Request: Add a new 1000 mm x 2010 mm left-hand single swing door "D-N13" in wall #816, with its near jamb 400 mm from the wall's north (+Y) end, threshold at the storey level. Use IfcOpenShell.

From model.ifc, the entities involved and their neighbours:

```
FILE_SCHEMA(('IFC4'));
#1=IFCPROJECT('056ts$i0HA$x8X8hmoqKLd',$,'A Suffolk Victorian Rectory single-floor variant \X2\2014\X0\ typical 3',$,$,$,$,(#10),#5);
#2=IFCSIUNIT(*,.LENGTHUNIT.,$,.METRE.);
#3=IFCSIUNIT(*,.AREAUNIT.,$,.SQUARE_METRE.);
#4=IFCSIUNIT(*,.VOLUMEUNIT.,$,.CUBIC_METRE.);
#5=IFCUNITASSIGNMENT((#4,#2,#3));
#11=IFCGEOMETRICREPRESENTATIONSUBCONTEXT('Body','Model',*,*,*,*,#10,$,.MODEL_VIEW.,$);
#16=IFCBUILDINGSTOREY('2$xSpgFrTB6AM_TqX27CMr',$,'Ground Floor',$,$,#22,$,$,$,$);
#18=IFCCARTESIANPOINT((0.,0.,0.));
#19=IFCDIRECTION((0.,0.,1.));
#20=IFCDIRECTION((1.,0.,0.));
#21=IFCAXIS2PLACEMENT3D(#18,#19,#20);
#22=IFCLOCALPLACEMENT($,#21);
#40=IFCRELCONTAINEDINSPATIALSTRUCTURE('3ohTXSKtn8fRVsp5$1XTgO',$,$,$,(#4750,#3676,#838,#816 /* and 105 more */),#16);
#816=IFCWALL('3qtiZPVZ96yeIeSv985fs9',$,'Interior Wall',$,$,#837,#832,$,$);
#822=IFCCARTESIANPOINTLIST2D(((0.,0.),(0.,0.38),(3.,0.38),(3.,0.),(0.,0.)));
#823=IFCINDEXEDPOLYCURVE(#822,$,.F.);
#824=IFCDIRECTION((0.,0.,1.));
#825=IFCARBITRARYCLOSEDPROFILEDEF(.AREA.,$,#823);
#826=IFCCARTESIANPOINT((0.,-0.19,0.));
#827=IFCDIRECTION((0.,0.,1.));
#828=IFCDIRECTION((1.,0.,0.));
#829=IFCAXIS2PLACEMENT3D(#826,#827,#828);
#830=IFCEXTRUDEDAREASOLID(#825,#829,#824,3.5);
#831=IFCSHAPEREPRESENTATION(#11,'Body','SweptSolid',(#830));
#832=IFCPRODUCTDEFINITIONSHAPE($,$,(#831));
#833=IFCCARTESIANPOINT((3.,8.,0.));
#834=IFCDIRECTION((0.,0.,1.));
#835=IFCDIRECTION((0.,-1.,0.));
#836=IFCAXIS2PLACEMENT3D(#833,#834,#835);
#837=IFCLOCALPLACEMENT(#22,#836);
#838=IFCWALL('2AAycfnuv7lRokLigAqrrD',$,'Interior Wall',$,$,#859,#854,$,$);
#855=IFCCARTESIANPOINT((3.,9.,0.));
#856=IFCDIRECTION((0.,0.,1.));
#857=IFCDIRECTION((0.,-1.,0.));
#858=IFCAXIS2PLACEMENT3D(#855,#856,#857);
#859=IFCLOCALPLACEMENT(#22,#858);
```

```python
import numpy as np
import ifcopenshell
import ifcopenshell.api.feature
import ifcopenshell.api.geometry
import ifcopenshell.api.root
import ifcopenshell.api.spatial
import ifcopenshell.geom
import ifcopenshell.util.element
import ifcopenshell.util.placement
import ifcopenshell.util.representation
import ifcopenshell.util.shape
import ifcopenshell.util.unit

model = ifcopenshell.open("model.ifc")
unit_scale = ifcopenshell.util.unit.calculate_unit_scale(model)
settings = ifcopenshell.geom.settings()


def volume(element):
    """Net volume in cubic metres, openings subtracted."""
    shape = ifcopenshell.geom.create_shape(settings, element)
    return ifcopenshell.util.shape.get_volume(shape.geometry)


wall = model.by_guid("3qtiZPVZ96yeIeSv985fs9")
storey = ifcopenshell.util.element.get_container(wall, ifc_class="IfcBuildingStorey")
context = ifcopenshell.util.representation.get_context(model, "Model", "Body", "MODEL_VIEW")
before = volume(wall)

width, height, from_end, sill = 1, 2.01, 0.4, 0.0  # metres

# The wall runs along its own X axis, and the end named is its -X end.
wall_shape = ifcopenshell.geom.create_shape(settings, wall)
x, y, z = ifcopenshell.util.shape.get_vertices(wall_shape.geometry).T
start = x.min() + from_end
face, thickness = float(y.min()), float(y.max() - y.min())
wall_matrix = ifcopenshell.util.placement.get_local_placement(wall.ObjectPlacement)
level = ifcopenshell.util.placement.get_local_placement(storey.ObjectPlacement)[2, 3]


def in_wall(x, y):
    """Placement at x, y metres in the wall's axes, at sill height."""
    matrix = wall_matrix.copy()
    matrix[:, 3] = wall_matrix @ np.array([x / unit_scale, y / unit_scale, 0.0, 1.0])
    matrix[2, 3] = level + sill / unit_scale
    return matrix


# Opening: a box that overshoots both wall faces by 50 mm.
opening = ifcopenshell.api.root.create_entity(model, ifc_class="IfcOpeningElement", predefined_type="OPENING")
box = ifcopenshell.api.geometry.add_wall_representation(
    model, context=context, length=width, height=height, thickness=thickness + 0.1
)
ifcopenshell.api.geometry.assign_representation(model, product=opening, representation=box)
ifcopenshell.api.geometry.edit_object_placement(model, product=opening, matrix=in_wall(start, face - 0.05), is_si=False)
ifcopenshell.api.feature.add_feature(model, feature=opening, element=wall)

door = ifcopenshell.api.root.create_entity(model, ifc_class="IfcDoor", name="D-N13", predefined_type="DOOR")
door.OverallWidth, door.OverallHeight = width / unit_scale, height / unit_scale
door.OperationType = "SINGLE_SWING_LEFT"
body = ifcopenshell.api.geometry.add_door_representation(
    model,
    context=context,
    overall_width=door.OverallWidth,
    overall_height=door.OverallHeight,
    operation_type="SINGLE_SWING_LEFT",
    lining_properties={"LiningDepth": thickness / unit_scale, "ThresholdDepth": thickness / unit_scale},
)
ifcopenshell.api.geometry.assign_representation(model, product=door, representation=body)
ifcopenshell.api.spatial.assign_container(model, products=[door], relating_structure=storey)
ifcopenshell.api.feature.add_filling(model, opening=opening, element=door)

# The lining spans the wall, so the door starts at the wall face.
ifcopenshell.api.geometry.edit_object_placement(model, product=door, matrix=in_wall(start, face), is_si=False)

after = volume(wall)

print(f"wall volume {before:.3f} -> {after:.3f} m3")

model.write("model-out.ifc")
```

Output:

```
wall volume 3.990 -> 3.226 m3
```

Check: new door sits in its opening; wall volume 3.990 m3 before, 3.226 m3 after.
